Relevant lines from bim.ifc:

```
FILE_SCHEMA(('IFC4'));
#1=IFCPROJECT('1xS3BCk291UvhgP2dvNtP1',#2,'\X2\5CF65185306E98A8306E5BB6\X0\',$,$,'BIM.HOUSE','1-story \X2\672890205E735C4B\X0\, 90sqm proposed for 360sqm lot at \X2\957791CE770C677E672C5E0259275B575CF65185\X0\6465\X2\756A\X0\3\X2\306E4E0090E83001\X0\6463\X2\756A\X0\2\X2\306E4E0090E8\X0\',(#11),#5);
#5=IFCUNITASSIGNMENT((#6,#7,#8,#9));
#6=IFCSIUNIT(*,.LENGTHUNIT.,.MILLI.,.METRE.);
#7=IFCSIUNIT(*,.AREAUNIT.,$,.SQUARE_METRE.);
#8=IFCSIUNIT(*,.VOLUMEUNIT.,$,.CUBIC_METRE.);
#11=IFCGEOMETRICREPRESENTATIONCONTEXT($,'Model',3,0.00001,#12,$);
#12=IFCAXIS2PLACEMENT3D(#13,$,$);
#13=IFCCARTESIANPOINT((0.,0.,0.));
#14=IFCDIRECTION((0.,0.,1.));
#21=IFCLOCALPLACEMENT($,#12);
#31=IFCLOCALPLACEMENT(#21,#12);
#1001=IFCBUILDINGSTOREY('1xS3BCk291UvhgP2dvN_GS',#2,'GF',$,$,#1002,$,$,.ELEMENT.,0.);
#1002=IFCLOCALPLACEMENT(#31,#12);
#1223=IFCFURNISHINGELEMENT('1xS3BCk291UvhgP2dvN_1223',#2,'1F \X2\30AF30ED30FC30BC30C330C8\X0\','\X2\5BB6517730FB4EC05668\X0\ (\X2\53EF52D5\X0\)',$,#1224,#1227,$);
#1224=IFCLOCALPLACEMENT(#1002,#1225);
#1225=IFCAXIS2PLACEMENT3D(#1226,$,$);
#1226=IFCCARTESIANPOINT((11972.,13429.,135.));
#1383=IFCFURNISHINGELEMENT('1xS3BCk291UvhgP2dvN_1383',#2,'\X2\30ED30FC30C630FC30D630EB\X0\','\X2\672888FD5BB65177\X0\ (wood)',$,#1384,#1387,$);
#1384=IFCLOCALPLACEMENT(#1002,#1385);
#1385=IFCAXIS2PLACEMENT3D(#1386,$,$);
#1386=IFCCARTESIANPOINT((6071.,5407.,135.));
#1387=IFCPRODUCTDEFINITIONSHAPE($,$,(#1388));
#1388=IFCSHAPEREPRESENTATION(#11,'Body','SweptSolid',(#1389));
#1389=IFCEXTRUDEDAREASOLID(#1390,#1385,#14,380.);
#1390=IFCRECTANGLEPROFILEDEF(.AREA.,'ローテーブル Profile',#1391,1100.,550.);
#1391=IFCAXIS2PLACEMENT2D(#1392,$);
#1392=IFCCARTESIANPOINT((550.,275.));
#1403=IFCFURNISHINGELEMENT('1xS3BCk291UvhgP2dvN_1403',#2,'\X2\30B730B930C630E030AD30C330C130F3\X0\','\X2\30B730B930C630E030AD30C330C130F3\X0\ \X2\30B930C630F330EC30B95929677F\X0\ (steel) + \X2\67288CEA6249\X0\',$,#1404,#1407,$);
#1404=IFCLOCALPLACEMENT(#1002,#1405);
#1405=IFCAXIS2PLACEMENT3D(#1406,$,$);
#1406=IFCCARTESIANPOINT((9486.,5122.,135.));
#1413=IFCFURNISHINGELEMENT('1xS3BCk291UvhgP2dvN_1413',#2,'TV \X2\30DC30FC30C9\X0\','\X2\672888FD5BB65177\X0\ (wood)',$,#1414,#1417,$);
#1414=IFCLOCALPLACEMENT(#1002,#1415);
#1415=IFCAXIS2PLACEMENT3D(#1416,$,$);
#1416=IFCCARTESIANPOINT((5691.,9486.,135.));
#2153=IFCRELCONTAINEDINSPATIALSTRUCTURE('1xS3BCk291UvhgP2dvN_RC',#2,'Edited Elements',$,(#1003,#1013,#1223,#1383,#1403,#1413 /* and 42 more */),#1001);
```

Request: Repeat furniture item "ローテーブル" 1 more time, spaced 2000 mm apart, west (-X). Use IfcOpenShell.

```python
import numpy as np
import ifcopenshell
import ifcopenshell.api.geometry
import ifcopenshell.api.root
import ifcopenshell.util.element
import ifcopenshell.util.placement

model = ifcopenshell.open("bim.ifc")


def reuse_history(source, copy):
    """copy_class also copies each property set's owner history, people and application; keep the originals."""
    for rel in copy.IsDefinedBy:
        if rel.is_a("IfcRelDefinesByProperties") and (history := rel.RelatingPropertyDefinition.OwnerHistory):
            rel.RelatingPropertyDefinition.OwnerHistory = source.OwnerHistory
            ifcopenshell.util.element.remove_deep2(model, history)


source = model.by_id(1383)
base = ifcopenshell.util.placement.get_local_placement(source.ObjectPlacement)
step = np.array([-1.0, 0.0, 0.0]) * 2000.0

for i in range(1, 2):
    copy = ifcopenshell.api.root.copy_class(model, product=source)
    copy.Representation = ifcopenshell.util.element.copy_deep(
        model, source.Representation, exclude=["IfcGeometricRepresentationContext", "IfcRepresentationMap"]
    )
    reuse_history(source, copy)
    matrix = base.copy()
    matrix[:3, 3] += i * step
    print("added at", matrix[:3, 3].round(3) + 0.0)
    ifcopenshell.api.geometry.edit_object_placement(model, product=copy, matrix=matrix, is_si=False)

model.write("bim_v2.ifc")
```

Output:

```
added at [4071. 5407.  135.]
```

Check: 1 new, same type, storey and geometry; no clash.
